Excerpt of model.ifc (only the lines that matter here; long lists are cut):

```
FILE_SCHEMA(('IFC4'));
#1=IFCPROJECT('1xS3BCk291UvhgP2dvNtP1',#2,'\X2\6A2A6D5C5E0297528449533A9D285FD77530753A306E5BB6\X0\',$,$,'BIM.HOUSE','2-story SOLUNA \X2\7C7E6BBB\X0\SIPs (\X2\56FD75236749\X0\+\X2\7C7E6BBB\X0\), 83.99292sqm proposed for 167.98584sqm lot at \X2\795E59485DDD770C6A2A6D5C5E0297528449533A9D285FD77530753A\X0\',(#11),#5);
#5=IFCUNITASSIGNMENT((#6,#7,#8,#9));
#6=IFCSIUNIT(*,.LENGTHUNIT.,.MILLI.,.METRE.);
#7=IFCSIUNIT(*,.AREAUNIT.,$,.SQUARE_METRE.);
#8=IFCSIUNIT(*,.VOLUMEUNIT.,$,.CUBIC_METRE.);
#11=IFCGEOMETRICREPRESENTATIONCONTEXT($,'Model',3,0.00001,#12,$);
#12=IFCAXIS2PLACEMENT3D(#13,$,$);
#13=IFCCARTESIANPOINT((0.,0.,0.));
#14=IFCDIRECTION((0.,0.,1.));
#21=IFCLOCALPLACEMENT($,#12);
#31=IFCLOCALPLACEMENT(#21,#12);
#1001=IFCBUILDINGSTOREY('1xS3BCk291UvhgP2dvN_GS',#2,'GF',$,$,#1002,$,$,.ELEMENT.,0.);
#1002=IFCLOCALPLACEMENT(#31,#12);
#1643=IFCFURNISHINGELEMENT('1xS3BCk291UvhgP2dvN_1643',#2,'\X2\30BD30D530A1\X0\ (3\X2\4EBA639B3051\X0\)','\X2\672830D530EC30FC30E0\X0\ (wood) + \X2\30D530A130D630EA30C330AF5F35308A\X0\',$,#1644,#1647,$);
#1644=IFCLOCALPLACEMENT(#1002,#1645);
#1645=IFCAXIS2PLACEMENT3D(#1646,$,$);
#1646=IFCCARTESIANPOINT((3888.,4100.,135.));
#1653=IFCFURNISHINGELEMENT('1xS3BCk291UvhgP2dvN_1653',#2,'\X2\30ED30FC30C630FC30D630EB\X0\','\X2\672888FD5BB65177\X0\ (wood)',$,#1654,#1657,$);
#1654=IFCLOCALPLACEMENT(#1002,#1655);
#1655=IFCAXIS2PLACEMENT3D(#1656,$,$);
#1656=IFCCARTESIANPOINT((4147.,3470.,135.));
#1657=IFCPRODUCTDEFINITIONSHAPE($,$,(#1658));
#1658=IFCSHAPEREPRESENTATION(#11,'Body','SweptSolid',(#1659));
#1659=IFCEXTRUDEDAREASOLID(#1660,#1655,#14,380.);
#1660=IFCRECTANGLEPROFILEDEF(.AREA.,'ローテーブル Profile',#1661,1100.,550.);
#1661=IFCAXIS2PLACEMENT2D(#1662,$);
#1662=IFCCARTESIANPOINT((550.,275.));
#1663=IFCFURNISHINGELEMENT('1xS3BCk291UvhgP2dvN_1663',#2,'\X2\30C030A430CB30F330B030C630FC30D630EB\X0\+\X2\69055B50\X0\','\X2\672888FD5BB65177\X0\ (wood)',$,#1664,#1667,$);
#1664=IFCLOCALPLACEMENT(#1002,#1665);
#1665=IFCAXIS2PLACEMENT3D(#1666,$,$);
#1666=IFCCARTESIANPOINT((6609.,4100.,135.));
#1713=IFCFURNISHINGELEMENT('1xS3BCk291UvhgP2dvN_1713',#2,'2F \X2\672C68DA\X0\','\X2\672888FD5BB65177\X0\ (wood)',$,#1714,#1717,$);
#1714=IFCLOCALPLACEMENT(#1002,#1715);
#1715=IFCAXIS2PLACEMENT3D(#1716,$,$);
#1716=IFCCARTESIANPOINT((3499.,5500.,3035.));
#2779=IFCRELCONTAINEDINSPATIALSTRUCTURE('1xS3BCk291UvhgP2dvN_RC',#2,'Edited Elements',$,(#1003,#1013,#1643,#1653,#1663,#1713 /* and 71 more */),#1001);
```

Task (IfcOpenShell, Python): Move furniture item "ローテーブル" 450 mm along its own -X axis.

```python
import ifcopenshell
import ifcopenshell.api.geometry
import ifcopenshell.util.placement

model = ifcopenshell.open("model.ifc")

item = model.by_id(1653)
matrix = ifcopenshell.util.placement.get_local_placement(item.ObjectPlacement)
matrix[:3, 3] -= matrix[:3, 0] * 450.0
ifcopenshell.api.geometry.edit_object_placement(model, product=item, matrix=matrix, is_si=False)

print(ifcopenshell.util.placement.get_local_placement(item.ObjectPlacement).round(3) + 0.0)

model.write("model_updated.ifc")
```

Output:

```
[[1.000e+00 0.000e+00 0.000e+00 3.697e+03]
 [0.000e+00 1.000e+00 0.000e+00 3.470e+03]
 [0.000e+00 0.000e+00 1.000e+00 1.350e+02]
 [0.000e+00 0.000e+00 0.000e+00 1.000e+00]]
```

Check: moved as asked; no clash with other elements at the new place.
